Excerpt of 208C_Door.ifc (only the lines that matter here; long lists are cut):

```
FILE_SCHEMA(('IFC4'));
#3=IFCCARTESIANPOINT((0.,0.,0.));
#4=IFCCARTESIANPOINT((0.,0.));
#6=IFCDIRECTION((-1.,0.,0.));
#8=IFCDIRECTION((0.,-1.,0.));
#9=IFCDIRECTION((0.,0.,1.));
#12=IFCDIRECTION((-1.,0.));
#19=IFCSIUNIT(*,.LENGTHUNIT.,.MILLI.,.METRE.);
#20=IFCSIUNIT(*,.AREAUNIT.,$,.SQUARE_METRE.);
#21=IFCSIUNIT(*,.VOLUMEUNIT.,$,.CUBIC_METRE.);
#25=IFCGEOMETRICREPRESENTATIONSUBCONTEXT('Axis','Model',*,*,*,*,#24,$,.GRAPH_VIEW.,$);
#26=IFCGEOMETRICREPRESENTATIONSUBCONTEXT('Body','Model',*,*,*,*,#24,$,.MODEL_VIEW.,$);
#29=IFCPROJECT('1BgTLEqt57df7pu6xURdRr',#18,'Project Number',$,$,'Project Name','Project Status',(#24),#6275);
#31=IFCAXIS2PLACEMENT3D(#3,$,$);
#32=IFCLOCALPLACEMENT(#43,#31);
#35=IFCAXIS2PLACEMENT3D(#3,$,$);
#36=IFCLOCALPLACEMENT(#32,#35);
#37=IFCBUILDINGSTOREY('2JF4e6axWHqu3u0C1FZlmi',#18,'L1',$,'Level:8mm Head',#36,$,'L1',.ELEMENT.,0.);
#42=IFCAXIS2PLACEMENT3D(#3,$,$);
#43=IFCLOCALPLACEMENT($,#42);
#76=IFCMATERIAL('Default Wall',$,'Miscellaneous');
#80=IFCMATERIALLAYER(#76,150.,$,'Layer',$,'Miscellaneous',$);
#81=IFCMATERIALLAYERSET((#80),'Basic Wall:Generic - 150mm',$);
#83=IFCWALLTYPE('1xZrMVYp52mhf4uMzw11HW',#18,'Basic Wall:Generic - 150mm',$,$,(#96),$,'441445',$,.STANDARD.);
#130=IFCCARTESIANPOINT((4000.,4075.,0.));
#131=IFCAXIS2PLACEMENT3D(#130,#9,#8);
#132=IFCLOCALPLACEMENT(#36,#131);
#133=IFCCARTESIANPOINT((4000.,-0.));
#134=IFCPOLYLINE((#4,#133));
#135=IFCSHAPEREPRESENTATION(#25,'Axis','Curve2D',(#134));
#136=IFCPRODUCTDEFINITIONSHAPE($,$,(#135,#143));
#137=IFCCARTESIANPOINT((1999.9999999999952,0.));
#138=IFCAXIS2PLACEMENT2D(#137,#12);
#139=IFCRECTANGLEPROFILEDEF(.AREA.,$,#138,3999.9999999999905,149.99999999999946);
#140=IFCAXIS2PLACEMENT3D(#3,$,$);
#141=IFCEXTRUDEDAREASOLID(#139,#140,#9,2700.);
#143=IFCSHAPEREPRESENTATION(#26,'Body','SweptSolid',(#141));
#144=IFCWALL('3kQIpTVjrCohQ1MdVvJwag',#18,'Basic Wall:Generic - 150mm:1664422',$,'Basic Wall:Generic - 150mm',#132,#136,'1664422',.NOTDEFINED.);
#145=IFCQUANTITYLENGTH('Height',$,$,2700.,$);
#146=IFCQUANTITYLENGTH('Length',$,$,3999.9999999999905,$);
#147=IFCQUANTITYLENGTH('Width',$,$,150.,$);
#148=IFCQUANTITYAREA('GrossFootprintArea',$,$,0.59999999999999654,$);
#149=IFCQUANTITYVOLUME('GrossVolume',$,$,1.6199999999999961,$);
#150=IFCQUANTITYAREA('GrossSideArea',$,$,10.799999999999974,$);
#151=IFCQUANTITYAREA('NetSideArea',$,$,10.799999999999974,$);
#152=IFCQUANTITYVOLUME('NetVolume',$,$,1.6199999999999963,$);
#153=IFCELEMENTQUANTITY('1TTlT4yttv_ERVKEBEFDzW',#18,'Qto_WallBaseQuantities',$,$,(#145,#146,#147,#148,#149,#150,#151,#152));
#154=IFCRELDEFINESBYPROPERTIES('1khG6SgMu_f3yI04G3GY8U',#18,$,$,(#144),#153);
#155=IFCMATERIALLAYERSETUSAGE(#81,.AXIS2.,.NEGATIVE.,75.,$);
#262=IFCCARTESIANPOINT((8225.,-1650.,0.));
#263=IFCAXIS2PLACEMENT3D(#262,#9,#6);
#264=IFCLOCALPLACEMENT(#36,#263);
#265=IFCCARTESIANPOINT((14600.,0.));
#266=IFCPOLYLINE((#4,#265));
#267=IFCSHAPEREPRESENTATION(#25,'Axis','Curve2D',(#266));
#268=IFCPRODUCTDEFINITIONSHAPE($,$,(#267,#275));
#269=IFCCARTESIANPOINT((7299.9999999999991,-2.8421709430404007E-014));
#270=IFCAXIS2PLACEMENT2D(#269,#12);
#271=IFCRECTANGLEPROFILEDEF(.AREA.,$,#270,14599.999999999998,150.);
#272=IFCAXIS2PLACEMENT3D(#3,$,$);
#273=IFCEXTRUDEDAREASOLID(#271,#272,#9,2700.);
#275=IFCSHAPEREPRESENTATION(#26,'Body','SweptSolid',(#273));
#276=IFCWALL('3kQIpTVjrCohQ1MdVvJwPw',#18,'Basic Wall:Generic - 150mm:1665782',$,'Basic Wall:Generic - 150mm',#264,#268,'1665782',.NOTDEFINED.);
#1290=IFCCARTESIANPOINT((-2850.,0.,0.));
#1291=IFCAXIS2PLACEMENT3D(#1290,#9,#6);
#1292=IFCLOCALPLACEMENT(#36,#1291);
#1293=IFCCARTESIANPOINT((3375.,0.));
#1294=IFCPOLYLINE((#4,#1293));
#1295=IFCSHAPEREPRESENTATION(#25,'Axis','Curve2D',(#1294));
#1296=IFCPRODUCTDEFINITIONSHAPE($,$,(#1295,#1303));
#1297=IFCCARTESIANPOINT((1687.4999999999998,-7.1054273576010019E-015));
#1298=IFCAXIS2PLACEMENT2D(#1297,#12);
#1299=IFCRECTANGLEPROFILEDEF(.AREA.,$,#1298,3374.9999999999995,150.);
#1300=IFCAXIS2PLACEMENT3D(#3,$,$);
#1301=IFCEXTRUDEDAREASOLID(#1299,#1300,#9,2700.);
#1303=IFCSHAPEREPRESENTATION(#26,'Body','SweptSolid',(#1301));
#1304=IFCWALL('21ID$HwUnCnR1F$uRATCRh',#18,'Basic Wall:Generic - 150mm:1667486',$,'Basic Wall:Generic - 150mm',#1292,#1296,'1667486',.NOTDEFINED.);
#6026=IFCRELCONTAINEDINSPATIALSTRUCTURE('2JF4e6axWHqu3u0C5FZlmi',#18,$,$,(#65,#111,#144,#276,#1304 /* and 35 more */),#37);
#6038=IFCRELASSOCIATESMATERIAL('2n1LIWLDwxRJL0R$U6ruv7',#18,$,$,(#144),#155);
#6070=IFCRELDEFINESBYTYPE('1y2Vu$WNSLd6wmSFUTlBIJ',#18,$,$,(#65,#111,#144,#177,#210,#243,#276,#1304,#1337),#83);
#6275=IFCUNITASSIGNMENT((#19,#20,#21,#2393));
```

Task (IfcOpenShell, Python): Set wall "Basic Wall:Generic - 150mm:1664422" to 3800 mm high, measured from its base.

```python
import ifcopenshell
import ifcopenshell.api.pset
import ifcopenshell.geom
import ifcopenshell.util.element
import ifcopenshell.util.representation
import ifcopenshell.util.shape
import ifcopenshell.util.unit

model = ifcopenshell.open("208C_Door.ifc")
unit_scale = ifcopenshell.util.unit.calculate_unit_scale(model)
area_scale = ifcopenshell.util.unit.calculate_unit_scale(model, "AREAUNIT")
volume_scale = ifcopenshell.util.unit.calculate_unit_scale(model, "VOLUMEUNIT")
settings = ifcopenshell.geom.settings()


def volume(element):
    """Net volume in cubic metres, openings subtracted."""
    shape = ifcopenshell.geom.create_shape(settings, element)
    return ifcopenshell.util.shape.get_volume(shape.geometry)


wall = model.by_id(144)
before = volume(wall)

body = ifcopenshell.util.representation.get_representation(wall, "Model", "Body")
solid = body.Items[0]
old_height = solid.Depth
solid.Depth = 3800.0
after = volume(wall)
thickness = 0.15  # wall thickness in metres

# Update the stored height, areas and volumes.
qto = model.by_id(ifcopenshell.util.element.get_pset(wall, "Qto_WallBaseQuantities", should_inherit=False)["id"])
ifcopenshell.api.pset.edit_qto(model, qto=qto, properties={
    "Height": solid.Depth,
    "GrossVolume": ifcopenshell.util.element.get_pset(wall, "Qto_WallBaseQuantities", "GrossVolume") * solid.Depth / old_height,
    "GrossSideArea": ifcopenshell.util.element.get_pset(wall, "Qto_WallBaseQuantities", "GrossSideArea") * solid.Depth / old_height,
    "NetSideArea": after / thickness / area_scale,
    "NetVolume": after / volume_scale,
})

print(f"height {old_height:g} -> {solid.Depth:g}, volume {before:.3f} -> {after:.3f} m3")

model.write("208C_Door_updated.ifc")
```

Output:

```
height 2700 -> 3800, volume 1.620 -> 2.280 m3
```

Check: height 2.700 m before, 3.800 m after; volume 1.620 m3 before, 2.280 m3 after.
